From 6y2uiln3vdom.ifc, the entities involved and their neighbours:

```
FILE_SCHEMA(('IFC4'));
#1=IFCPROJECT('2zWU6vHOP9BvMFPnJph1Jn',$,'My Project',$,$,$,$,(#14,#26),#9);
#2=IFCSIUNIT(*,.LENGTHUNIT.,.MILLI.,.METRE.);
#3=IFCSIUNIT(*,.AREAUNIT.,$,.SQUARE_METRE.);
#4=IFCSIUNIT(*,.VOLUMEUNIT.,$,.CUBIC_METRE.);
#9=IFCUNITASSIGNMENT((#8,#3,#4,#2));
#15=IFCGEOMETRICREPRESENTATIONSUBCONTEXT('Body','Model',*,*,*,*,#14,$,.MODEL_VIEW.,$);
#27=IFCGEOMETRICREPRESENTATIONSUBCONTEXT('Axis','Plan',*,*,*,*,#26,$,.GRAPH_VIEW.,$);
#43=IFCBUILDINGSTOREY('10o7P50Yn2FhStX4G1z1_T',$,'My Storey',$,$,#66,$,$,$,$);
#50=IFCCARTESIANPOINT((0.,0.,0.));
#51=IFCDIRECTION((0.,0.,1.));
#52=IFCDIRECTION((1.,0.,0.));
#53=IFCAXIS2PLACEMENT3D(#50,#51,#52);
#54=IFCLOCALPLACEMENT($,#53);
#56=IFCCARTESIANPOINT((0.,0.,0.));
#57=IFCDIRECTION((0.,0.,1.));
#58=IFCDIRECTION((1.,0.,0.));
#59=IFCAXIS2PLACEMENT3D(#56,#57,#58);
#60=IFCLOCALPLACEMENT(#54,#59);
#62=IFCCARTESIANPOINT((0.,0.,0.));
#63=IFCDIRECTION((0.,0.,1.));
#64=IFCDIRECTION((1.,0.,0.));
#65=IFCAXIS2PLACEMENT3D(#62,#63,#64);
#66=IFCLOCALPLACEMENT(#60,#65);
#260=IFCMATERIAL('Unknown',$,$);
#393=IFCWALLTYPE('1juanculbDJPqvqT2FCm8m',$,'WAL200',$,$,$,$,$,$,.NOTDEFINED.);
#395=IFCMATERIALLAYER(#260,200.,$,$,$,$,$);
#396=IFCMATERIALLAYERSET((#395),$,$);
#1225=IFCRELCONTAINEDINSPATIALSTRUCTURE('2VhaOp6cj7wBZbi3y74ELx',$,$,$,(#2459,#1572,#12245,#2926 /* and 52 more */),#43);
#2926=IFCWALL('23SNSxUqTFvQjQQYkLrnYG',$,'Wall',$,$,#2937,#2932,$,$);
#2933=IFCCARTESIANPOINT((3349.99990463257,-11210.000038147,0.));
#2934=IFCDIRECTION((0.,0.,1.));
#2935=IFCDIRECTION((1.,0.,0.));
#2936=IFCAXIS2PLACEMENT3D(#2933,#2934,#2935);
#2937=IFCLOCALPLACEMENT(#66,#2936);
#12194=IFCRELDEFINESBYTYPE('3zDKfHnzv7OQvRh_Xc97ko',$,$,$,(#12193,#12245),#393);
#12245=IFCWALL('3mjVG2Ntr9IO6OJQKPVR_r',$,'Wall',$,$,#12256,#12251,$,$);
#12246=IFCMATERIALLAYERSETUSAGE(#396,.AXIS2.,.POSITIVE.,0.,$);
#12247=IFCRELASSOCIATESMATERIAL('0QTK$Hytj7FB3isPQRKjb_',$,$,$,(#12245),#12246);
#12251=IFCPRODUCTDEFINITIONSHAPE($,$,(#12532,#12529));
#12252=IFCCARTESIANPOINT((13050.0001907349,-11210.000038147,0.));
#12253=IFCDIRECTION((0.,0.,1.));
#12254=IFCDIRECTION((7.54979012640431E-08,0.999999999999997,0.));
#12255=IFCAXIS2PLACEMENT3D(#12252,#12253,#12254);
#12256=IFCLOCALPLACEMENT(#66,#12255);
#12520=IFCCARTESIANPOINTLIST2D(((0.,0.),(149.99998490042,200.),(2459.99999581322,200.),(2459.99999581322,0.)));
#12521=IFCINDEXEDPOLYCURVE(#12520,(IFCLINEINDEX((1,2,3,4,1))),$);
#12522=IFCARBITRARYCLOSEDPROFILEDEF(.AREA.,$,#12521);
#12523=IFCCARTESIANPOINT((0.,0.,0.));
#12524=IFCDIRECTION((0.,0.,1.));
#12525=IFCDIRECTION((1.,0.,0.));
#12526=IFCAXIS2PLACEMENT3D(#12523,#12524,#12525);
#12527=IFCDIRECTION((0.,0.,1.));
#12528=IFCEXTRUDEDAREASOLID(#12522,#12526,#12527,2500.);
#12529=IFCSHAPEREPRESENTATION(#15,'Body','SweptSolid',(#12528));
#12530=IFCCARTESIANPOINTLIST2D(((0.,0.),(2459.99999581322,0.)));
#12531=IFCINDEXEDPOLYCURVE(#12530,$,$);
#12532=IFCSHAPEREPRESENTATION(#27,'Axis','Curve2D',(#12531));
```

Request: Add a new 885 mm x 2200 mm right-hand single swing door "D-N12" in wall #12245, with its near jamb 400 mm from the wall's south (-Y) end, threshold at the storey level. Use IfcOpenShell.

```python
import numpy as np
import ifcopenshell
import ifcopenshell.api.feature
import ifcopenshell.api.geometry
import ifcopenshell.api.root
import ifcopenshell.api.spatial
import ifcopenshell.geom
import ifcopenshell.util.element
import ifcopenshell.util.placement
import ifcopenshell.util.representation
import ifcopenshell.util.shape
import ifcopenshell.util.unit

model = ifcopenshell.open("6y2uiln3vdom.ifc")
unit_scale = ifcopenshell.util.unit.calculate_unit_scale(model)
settings = ifcopenshell.geom.settings()


def volume(element):
    """Net volume in cubic metres, openings subtracted."""
    shape = ifcopenshell.geom.create_shape(settings, element)
    return ifcopenshell.util.shape.get_volume(shape.geometry)


wall = model.by_id(12245)
storey = ifcopenshell.util.element.get_container(wall, ifc_class="IfcBuildingStorey")
context = ifcopenshell.util.representation.get_context(model, "Model", "Body", "MODEL_VIEW")
before = volume(wall)

width, height, from_end, sill = 0.885, 2.2, 0.4, 0.0  # metres

# The wall runs along its own X axis, and the end named is its -X end.
wall_shape = ifcopenshell.geom.create_shape(settings, wall)
x, y, z = ifcopenshell.util.shape.get_vertices(wall_shape.geometry).T
start = x.min() + from_end
face, thickness = float(y.min()), float(y.max() - y.min())
wall_matrix = ifcopenshell.util.placement.get_local_placement(wall.ObjectPlacement)
level = ifcopenshell.util.placement.get_local_placement(storey.ObjectPlacement)[2, 3]


def in_wall(x, y):
    """Placement at x, y metres in the wall's axes, at sill height."""
    matrix = wall_matrix.copy()
    matrix[:, 3] = wall_matrix @ np.array([x / unit_scale, y / unit_scale, 0.0, 1.0])
    matrix[2, 3] = level + sill / unit_scale
    return matrix


# Opening: a box that overshoots both wall faces by 50 mm.
opening = ifcopenshell.api.root.create_entity(model, ifc_class="IfcOpeningElement", predefined_type="OPENING")
box = ifcopenshell.api.geometry.add_wall_representation(
    model, context=context, length=width, height=height, thickness=thickness + 0.1
)
ifcopenshell.api.geometry.assign_representation(model, product=opening, representation=box)
ifcopenshell.api.geometry.edit_object_placement(model, product=opening, matrix=in_wall(start, face - 0.05), is_si=False)
ifcopenshell.api.feature.add_feature(model, feature=opening, element=wall)

door = ifcopenshell.api.root.create_entity(model, ifc_class="IfcDoor", name="D-N12", predefined_type="DOOR")
door.OverallWidth, door.OverallHeight = width / unit_scale, height / unit_scale
door.OperationType = "SINGLE_SWING_RIGHT"
body = ifcopenshell.api.geometry.add_door_representation(
    model,
    context=context,
    overall_width=door.OverallWidth,
    overall_height=door.OverallHeight,
    operation_type="SINGLE_SWING_RIGHT",
    lining_properties={"LiningDepth": thickness / unit_scale, "ThresholdDepth": thickness / unit_scale},
)
ifcopenshell.api.geometry.assign_representation(model, product=door, representation=body)
ifcopenshell.api.spatial.assign_container(model, products=[door], relating_structure=storey)
ifcopenshell.api.feature.add_filling(model, opening=opening, element=door)

# The lining spans the wall, so the door starts at the wall face.
ifcopenshell.api.geometry.edit_object_placement(model, product=door, matrix=in_wall(start, face), is_si=False)

after = volume(wall)

print(f"wall volume {before:.3f} -> {after:.3f} m3")

model.write("6y2uiln3vdom_updated.ifc")
```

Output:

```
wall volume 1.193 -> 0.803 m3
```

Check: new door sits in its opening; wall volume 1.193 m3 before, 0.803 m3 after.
